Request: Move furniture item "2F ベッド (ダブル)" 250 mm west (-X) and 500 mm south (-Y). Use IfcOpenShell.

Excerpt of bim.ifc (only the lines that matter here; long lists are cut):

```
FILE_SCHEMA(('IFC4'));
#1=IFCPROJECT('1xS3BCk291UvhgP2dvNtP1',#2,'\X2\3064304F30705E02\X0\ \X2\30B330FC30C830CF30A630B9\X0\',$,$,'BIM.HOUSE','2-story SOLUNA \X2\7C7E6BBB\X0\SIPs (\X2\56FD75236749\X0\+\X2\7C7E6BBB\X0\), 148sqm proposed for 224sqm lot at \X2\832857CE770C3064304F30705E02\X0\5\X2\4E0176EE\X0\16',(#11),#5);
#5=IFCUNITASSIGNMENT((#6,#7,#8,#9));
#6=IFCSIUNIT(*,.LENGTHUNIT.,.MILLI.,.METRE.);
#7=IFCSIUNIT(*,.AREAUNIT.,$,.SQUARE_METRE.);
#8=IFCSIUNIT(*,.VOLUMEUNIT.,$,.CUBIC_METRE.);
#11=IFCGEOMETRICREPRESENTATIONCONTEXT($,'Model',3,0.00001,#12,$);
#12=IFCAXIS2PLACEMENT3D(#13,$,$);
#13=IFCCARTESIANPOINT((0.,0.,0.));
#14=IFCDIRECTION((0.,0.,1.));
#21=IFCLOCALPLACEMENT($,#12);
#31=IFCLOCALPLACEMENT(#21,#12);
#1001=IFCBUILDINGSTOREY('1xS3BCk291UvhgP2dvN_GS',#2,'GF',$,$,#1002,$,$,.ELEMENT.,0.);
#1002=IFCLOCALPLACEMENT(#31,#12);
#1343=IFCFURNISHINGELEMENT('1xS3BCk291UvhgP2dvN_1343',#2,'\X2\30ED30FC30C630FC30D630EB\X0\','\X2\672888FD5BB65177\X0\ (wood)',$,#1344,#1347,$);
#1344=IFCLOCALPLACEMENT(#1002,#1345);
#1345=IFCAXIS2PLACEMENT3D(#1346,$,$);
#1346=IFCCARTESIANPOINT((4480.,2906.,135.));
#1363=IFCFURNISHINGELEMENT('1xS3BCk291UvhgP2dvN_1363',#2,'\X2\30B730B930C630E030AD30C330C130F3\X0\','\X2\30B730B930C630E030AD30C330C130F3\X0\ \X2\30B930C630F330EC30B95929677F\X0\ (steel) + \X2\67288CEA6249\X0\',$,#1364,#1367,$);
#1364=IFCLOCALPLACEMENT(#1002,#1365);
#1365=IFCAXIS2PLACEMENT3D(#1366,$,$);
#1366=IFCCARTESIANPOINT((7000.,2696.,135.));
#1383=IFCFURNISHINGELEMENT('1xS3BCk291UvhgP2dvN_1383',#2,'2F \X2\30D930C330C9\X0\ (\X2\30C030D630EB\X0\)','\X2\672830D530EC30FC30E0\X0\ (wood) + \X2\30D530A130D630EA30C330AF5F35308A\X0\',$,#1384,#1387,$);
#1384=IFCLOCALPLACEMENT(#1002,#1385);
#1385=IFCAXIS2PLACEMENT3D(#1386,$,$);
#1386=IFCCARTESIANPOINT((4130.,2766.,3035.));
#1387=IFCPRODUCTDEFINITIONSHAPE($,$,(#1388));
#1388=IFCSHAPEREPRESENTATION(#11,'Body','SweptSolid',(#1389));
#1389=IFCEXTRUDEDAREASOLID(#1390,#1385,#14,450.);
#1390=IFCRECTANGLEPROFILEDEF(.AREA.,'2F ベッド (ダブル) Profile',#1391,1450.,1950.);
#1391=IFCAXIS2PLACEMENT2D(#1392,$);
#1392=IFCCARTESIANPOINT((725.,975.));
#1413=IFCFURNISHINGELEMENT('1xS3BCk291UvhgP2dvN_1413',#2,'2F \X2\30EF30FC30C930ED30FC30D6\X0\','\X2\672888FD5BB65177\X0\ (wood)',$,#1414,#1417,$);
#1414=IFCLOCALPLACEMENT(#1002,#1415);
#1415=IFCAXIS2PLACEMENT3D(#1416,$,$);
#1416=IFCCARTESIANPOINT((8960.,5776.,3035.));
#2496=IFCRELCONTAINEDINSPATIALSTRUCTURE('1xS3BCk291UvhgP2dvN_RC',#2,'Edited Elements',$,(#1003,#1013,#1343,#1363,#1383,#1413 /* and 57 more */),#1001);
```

```python
import ifcopenshell
import ifcopenshell.api.geometry
import ifcopenshell.util.placement
import ifcopenshell.util.unit

model = ifcopenshell.open("bim.ifc")
unit_scale = ifcopenshell.util.unit.calculate_unit_scale(model)

item = model.by_guid("1xS3BCk291UvhgP2dvN_1383")
matrix = ifcopenshell.util.placement.get_local_placement(item.ObjectPlacement)
matrix[0, 3] -= 0.25 / unit_scale
matrix[1, 3] -= 0.5 / unit_scale
ifcopenshell.api.geometry.edit_object_placement(model, product=item, matrix=matrix, is_si=False)

print(ifcopenshell.util.placement.get_local_placement(item.ObjectPlacement).round(3) + 0.0)

model.write("bim-out.ifc")
```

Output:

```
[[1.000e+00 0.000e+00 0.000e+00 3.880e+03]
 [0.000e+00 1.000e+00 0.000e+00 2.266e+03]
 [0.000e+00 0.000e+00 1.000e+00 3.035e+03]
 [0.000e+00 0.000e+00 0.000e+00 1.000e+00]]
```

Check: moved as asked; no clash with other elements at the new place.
